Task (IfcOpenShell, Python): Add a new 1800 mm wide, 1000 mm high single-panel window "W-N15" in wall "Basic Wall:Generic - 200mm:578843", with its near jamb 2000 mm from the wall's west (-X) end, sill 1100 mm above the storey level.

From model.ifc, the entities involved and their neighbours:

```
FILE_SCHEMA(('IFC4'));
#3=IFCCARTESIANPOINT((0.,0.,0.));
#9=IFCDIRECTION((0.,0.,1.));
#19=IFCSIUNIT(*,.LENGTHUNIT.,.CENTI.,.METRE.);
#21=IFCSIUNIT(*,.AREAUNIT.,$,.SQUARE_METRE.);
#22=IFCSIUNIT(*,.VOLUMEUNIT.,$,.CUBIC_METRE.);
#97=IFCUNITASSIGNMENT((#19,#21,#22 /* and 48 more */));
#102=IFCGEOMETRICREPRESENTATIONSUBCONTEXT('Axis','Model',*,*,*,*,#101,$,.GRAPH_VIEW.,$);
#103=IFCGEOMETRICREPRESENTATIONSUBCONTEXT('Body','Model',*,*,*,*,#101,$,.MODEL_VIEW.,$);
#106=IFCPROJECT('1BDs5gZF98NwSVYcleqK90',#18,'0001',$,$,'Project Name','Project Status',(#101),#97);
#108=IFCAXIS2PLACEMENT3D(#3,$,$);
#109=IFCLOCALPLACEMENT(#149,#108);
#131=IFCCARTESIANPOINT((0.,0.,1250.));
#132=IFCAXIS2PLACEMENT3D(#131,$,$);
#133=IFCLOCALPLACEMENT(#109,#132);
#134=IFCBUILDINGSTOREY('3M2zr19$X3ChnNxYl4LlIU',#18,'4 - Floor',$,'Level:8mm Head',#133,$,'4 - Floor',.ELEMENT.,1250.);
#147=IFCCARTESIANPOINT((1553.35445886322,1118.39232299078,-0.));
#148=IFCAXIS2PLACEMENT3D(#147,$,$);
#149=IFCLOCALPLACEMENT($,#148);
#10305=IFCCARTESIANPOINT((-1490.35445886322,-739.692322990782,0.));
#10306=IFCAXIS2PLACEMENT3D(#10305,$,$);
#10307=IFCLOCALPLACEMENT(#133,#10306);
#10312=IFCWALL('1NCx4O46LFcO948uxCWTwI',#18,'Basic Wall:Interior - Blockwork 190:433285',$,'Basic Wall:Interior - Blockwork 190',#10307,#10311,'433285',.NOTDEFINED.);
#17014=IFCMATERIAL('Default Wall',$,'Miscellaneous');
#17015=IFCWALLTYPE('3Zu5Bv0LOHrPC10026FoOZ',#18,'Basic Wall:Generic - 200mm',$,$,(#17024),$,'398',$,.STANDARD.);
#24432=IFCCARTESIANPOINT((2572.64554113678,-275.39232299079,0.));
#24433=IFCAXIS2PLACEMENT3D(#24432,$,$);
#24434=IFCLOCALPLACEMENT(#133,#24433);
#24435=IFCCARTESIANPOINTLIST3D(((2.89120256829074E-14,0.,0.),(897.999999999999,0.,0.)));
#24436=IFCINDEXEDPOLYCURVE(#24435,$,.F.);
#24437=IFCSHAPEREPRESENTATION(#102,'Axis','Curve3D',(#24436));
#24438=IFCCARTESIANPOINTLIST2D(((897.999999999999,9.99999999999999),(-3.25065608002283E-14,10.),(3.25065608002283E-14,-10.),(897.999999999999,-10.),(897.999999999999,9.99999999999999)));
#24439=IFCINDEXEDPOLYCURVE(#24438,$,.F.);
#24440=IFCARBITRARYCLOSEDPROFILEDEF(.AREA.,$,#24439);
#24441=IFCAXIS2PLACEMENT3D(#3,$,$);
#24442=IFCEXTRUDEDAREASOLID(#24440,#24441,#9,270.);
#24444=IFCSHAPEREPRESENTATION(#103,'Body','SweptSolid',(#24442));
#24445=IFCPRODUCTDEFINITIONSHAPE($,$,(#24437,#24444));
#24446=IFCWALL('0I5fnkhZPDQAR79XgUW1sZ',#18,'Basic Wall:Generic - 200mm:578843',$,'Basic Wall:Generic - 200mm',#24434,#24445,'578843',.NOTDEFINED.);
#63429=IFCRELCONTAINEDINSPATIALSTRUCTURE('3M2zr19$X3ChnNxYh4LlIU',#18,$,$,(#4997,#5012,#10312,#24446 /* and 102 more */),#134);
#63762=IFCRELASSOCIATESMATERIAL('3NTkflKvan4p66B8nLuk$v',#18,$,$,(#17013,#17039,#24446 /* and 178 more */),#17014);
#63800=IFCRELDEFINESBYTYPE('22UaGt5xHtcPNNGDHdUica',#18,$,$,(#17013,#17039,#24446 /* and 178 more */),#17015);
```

```python
import numpy as np
import ifcopenshell
import ifcopenshell.api.feature
import ifcopenshell.api.geometry
import ifcopenshell.api.root
import ifcopenshell.api.spatial
import ifcopenshell.geom
import ifcopenshell.util.element
import ifcopenshell.util.placement
import ifcopenshell.util.representation
import ifcopenshell.util.shape
import ifcopenshell.util.unit

model = ifcopenshell.open("model.ifc")
unit_scale = ifcopenshell.util.unit.calculate_unit_scale(model)
settings = ifcopenshell.geom.settings()


def volume(element):
    """Net volume in cubic metres, openings subtracted."""
    shape = ifcopenshell.geom.create_shape(settings, element)
    return ifcopenshell.util.shape.get_volume(shape.geometry)


wall = model.by_guid("0I5fnkhZPDQAR79XgUW1sZ")
storey = ifcopenshell.util.element.get_container(wall, ifc_class="IfcBuildingStorey")
context = ifcopenshell.util.representation.get_context(model, "Model", "Body", "MODEL_VIEW")
before = volume(wall)

width, height, from_end, sill = 1.8, 1, 2, 1.1  # metres

# The wall runs along its own X axis, and the end named is its -X end.
wall_shape = ifcopenshell.geom.create_shape(settings, wall)
x, y, z = ifcopenshell.util.shape.get_vertices(wall_shape.geometry).T
start = x.min() + from_end
face, thickness = float(y.min()), float(y.max() - y.min())
wall_matrix = ifcopenshell.util.placement.get_local_placement(wall.ObjectPlacement)
level = ifcopenshell.util.placement.get_local_placement(storey.ObjectPlacement)[2, 3]


def in_wall(x, y):
    """Placement at x, y metres in the wall's axes, at sill height."""
    matrix = wall_matrix.copy()
    matrix[:, 3] = wall_matrix @ np.array([x / unit_scale, y / unit_scale, 0.0, 1.0])
    matrix[2, 3] = level + sill / unit_scale
    return matrix


# Opening: a box that overshoots both wall faces by 50 mm.
opening = ifcopenshell.api.root.create_entity(model, ifc_class="IfcOpeningElement", predefined_type="OPENING")
box = ifcopenshell.api.geometry.add_wall_representation(
    model, context=context, length=width, height=height, thickness=thickness + 0.1
)
ifcopenshell.api.geometry.assign_representation(model, product=opening, representation=box)
ifcopenshell.api.geometry.edit_object_placement(model, product=opening, matrix=in_wall(start, face - 0.05), is_si=False)
ifcopenshell.api.feature.add_feature(model, feature=opening, element=wall)

window = ifcopenshell.api.root.create_entity(model, ifc_class="IfcWindow", name="W-N15", predefined_type="WINDOW")
window.OverallWidth, window.OverallHeight = width / unit_scale, height / unit_scale
window.PartitioningType = "SINGLE_PANEL"
body = ifcopenshell.api.geometry.add_window_representation(
    model,
    context=context,
    overall_width=window.OverallWidth,
    overall_height=window.OverallHeight,
    partition_type="SINGLE_PANEL",
)
ifcopenshell.api.geometry.assign_representation(model, product=window, representation=body)
ifcopenshell.api.spatial.assign_container(model, products=[window], relating_structure=storey)
ifcopenshell.api.feature.add_filling(model, opening=opening, element=window)

# Centre the window in the wall's thickness.
ifcopenshell.api.geometry.edit_object_placement(model, product=window, matrix=in_wall(start, face), is_si=False)
window_shape = ifcopenshell.geom.create_shape(settings, window)
depth = ifcopenshell.util.shape.get_vertices(window_shape.geometry)[:, 1]
offset = face + thickness / 2 - (depth.min() + depth.max()) / 2
ifcopenshell.api.geometry.edit_object_placement(model, product=window, matrix=in_wall(start, offset), is_si=False)

after = volume(wall)

print(f"wall volume {before:.3f} -> {after:.3f} m3")

model.write("model_v2.ifc")
```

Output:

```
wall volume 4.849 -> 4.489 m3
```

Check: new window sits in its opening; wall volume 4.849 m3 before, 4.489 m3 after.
